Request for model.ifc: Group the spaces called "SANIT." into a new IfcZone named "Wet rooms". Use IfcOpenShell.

First a look at what the model holds.

```python
import ifcopenshell

model = ifcopenshell.open("model.ifc")
print(model.schema)
seen = {}
for space in model.by_type("IfcSpace"):
    seen[space.LongName] = seen.get(space.LongName, 0) + 1
for name, count in sorted(seen.items(), key=str):
    print(count, "x", name)
print("zones:", [z.Name for z in model.by_type("IfcZone")][:20])
```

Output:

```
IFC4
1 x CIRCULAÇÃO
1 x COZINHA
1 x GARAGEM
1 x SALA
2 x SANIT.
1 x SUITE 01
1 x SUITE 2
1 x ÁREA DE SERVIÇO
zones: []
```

```python
import ifcopenshell
import ifcopenshell.api.group
import ifcopenshell.api.root

model = ifcopenshell.open("model.ifc")

names = {"SANIT."}
spaces = [s for s in model.by_type("IfcSpace") if s.LongName in names]

zone = ifcopenshell.api.root.create_entity(model, ifc_class="IfcZone", name="Wet rooms")
ifcopenshell.api.group.assign_group(model, products=spaces, group=zone)
print(len(spaces), "spaces in", zone.Name)

model.write("model_updated.ifc")
```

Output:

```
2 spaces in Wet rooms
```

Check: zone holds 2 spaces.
